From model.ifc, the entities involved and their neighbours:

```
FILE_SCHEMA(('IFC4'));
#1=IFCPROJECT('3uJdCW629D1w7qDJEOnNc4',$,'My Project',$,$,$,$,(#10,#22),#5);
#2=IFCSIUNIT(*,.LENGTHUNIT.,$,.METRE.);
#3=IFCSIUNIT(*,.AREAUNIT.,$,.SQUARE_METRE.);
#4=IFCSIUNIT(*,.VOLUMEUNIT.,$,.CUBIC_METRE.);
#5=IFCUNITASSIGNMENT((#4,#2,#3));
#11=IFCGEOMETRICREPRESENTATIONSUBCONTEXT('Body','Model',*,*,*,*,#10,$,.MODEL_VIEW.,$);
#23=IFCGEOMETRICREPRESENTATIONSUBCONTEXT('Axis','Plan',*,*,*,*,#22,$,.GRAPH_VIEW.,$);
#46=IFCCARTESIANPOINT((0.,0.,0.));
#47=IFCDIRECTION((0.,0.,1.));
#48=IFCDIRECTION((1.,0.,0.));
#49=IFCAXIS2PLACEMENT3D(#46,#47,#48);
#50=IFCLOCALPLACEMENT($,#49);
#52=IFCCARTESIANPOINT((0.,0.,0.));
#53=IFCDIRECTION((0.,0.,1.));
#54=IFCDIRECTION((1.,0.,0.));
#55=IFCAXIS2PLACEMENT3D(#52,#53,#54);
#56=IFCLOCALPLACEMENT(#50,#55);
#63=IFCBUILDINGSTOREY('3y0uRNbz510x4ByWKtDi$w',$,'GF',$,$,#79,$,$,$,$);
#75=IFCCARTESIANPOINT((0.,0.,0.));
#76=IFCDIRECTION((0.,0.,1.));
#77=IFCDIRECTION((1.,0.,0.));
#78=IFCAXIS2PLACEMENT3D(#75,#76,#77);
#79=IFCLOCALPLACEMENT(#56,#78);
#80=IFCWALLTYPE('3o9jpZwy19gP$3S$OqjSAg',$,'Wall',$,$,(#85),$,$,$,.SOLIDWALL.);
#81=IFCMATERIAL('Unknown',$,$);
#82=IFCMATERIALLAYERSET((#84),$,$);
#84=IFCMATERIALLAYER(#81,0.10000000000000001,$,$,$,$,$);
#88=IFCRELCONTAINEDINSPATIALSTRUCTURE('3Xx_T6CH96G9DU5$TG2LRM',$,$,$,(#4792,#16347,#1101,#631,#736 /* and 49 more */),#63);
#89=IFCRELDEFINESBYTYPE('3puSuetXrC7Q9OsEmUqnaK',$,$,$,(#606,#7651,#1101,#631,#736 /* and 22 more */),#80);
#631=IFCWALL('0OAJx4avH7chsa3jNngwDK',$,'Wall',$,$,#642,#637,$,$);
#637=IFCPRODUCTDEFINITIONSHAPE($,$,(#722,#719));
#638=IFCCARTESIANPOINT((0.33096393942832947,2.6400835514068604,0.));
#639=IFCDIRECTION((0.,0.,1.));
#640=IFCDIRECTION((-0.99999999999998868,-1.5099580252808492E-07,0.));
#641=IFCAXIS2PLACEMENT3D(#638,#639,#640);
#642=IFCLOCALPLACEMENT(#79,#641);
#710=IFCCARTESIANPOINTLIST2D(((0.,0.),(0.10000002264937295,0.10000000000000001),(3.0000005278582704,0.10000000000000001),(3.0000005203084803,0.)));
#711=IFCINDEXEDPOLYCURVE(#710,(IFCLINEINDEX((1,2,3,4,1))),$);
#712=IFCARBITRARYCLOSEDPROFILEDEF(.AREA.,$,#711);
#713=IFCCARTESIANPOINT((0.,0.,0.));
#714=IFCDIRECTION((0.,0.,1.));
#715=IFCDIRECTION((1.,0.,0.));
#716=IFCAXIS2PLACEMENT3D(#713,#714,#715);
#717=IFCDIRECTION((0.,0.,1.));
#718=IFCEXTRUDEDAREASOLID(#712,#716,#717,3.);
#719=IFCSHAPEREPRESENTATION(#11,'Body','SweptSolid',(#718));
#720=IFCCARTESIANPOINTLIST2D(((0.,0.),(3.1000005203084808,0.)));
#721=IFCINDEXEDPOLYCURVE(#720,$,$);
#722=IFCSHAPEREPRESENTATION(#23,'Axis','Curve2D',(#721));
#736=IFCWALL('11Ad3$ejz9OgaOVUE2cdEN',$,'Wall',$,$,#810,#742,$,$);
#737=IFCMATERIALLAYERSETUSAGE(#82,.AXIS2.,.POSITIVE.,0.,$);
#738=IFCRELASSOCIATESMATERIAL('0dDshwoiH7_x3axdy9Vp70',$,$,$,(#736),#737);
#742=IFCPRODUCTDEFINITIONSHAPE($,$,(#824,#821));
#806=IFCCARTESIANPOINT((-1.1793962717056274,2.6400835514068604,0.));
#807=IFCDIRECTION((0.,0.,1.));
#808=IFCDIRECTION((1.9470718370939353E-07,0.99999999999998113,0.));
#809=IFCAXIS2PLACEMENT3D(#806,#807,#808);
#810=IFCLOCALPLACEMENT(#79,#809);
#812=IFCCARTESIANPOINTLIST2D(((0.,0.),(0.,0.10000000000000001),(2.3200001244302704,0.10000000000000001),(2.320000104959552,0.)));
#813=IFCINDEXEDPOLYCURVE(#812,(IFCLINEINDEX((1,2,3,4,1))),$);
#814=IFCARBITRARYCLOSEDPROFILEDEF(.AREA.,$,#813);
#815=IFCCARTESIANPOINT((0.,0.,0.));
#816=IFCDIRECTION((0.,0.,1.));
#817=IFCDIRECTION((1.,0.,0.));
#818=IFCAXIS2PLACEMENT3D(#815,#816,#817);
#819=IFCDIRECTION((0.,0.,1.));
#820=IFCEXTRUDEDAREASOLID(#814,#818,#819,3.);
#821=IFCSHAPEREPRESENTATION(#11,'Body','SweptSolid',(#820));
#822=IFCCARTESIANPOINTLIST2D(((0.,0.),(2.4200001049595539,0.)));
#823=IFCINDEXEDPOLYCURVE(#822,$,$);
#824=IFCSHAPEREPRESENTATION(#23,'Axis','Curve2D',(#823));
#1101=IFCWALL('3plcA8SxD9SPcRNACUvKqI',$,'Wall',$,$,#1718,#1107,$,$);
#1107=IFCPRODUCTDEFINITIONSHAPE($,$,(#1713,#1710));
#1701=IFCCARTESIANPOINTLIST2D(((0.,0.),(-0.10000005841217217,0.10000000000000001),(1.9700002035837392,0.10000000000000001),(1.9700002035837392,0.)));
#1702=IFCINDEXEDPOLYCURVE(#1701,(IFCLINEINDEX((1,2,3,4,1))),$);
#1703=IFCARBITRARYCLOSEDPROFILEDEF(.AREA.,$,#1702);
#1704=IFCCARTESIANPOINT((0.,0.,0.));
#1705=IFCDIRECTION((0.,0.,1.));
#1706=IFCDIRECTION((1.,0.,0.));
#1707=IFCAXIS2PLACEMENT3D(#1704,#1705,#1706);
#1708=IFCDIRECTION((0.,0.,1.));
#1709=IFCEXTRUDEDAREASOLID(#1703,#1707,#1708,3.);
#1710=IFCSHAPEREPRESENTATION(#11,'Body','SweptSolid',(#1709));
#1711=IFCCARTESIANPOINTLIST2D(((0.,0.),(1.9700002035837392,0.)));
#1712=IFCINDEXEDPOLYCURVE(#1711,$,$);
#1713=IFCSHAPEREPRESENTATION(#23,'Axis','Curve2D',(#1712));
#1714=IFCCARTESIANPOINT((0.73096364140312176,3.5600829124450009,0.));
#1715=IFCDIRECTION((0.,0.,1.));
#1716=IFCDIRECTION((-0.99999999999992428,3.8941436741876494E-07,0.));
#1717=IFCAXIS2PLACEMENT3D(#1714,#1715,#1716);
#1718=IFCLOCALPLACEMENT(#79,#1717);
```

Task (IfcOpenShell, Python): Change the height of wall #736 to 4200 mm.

```python
import ifcopenshell
import ifcopenshell.geom
import ifcopenshell.util.representation
import ifcopenshell.util.shape

model = ifcopenshell.open("model.ifc")
settings = ifcopenshell.geom.settings()


def volume(element):
    """Net volume in cubic metres, openings subtracted."""
    shape = ifcopenshell.geom.create_shape(settings, element)
    return ifcopenshell.util.shape.get_volume(shape.geometry)


wall = model.by_guid("11Ad3$ejz9OgaOVUE2cdEN")
before = volume(wall)

body = ifcopenshell.util.representation.get_representation(wall, "Model", "Body")
solid = body.Items[0]
old_height = solid.Depth
solid.Depth = 4.2
after = volume(wall)

print(f"height {old_height:g} -> {solid.Depth:g}, volume {before:.3f} -> {after:.3f} m3")

model.write("model_v2.ifc")
```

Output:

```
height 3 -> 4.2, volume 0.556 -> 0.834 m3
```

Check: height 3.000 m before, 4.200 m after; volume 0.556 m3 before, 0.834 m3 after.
